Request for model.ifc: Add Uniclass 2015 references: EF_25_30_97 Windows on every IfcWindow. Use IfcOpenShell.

First a look at what the model holds.

```python
import ifcopenshell

model = ifcopenshell.open("model.ifc")
print(model.schema)
print("classifications:", [c.Name for c in model.by_type("IfcClassification")])
for ifc_class in ("IfcDoor", "IfcRoof", "IfcStair", "IfcWall", "IfcWindow"):
    print(ifc_class, len(model.by_type(ifc_class)))
```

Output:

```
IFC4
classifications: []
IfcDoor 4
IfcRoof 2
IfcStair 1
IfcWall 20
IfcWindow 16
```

```python
import ifcopenshell
import ifcopenshell.api.classification

model = ifcopenshell.open("model.ifc")

system = ifcopenshell.api.classification.add_classification(model, classification="Uniclass 2015")

codes = {
    "IfcWindow": ("EF_25_30_97", "Windows"),
}
for ifc_class, (code, name) in codes.items():
    products = model.by_type(ifc_class)
    ifcopenshell.api.classification.add_reference(
        model, products=products, classification=system, identification=code, name=name
    )
    print(code, len(products))

model.write("model_edited.ifc")
```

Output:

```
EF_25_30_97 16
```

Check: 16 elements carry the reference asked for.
